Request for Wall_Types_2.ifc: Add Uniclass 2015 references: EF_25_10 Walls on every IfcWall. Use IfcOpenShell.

First a look at what the model holds.

```python
import ifcopenshell

model = ifcopenshell.open("Wall_Types_2.ifc")
print(model.schema)
print("classifications:", [c.Name for c in model.by_type("IfcClassification")])
for ifc_class in ("IfcDoor", "IfcRoof", "IfcStair", "IfcWall", "IfcWindow"):
    print(ifc_class, len(model.by_type(ifc_class)))
```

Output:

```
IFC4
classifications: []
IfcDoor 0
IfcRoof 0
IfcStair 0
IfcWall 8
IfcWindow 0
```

```python
import ifcopenshell
import ifcopenshell.api.classification

model = ifcopenshell.open("Wall_Types_2.ifc")

system = ifcopenshell.api.classification.add_classification(model, classification="Uniclass 2015")

codes = {
    "IfcWall": ("EF_25_10", "Walls"),
}
for ifc_class, (code, name) in codes.items():
    products = model.by_type(ifc_class)
    ifcopenshell.api.classification.add_reference(
        model, products=products, classification=system, identification=code, name=name
    )
    print(code, len(products))

model.write("Wall_Types_2_updated.ifc")
```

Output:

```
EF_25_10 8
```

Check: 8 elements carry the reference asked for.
